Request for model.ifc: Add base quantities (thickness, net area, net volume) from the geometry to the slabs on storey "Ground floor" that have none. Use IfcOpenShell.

First a look at what the model holds.

```python
import ifcopenshell
import ifcopenshell.util.element
import ifcopenshell.util.unit

model = ifcopenshell.open("model.ifc")
print(model.schema)
for unit_type in ("LENGTHUNIT", "AREAUNIT", "VOLUMEUNIT"):
    print(unit_type, ifcopenshell.util.unit.calculate_unit_scale(model, unit_type))
storey = next(s for s in model.by_type("IfcBuildingStorey") if s.Name == "Ground floor")
slabs = [e for e in ifcopenshell.util.element.get_decomposition(storey) if e.is_a("IfcSlab")]
for e in sorted(slabs, key=lambda e: e.id()):
    print(e.id(), e.is_a(), e.Name, list(ifcopenshell.util.element.get_psets(e, qtos_only=True)), sep=" | ")
```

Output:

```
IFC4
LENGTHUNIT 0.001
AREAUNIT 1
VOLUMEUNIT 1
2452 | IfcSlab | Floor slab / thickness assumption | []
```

```python
import ifcopenshell
import ifcopenshell.api.pset
import ifcopenshell.geom
import ifcopenshell.util.element
import ifcopenshell.util.shape
import ifcopenshell.util.unit

model = ifcopenshell.open("model.ifc")
unit_scale = ifcopenshell.util.unit.calculate_unit_scale(model)
area_scale = ifcopenshell.util.unit.calculate_unit_scale(model, "AREAUNIT")
volume_scale = ifcopenshell.util.unit.calculate_unit_scale(model, "VOLUMEUNIT")
settings = ifcopenshell.geom.settings()

storey = next(s for s in model.by_type("IfcBuildingStorey") if s.Name == "Ground floor")
slabs = [e for e in ifcopenshell.util.element.get_decomposition(storey) if e.is_a("IfcSlab")]

for e in sorted(slabs, key=lambda e: e.id()):
    if ifcopenshell.util.element.get_psets(e, qtos_only=True, should_inherit=False):
        continue
    # Geometry comes back in metres, in the element's own axes.
    shape = ifcopenshell.geom.create_shape(settings, e)
    values = {
        "Width": ifcopenshell.util.shape.get_z(shape.geometry) / unit_scale,
        "NetArea": ifcopenshell.util.shape.get_footprint_area(shape.geometry) / area_scale,
        "NetVolume": ifcopenshell.util.shape.get_volume(shape.geometry) / volume_scale,
    }
    qto = ifcopenshell.api.pset.add_qto(model, product=e, name="Qto_SlabBaseQuantities")
    ifcopenshell.api.pset.edit_qto(model, qto=qto, properties=values)
    print(e.id(), {k: round(v, 3) for k, v in values.items()})

model.write("model_v2.ifc")
```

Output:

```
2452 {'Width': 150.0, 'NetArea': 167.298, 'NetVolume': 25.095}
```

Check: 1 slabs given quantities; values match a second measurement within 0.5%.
